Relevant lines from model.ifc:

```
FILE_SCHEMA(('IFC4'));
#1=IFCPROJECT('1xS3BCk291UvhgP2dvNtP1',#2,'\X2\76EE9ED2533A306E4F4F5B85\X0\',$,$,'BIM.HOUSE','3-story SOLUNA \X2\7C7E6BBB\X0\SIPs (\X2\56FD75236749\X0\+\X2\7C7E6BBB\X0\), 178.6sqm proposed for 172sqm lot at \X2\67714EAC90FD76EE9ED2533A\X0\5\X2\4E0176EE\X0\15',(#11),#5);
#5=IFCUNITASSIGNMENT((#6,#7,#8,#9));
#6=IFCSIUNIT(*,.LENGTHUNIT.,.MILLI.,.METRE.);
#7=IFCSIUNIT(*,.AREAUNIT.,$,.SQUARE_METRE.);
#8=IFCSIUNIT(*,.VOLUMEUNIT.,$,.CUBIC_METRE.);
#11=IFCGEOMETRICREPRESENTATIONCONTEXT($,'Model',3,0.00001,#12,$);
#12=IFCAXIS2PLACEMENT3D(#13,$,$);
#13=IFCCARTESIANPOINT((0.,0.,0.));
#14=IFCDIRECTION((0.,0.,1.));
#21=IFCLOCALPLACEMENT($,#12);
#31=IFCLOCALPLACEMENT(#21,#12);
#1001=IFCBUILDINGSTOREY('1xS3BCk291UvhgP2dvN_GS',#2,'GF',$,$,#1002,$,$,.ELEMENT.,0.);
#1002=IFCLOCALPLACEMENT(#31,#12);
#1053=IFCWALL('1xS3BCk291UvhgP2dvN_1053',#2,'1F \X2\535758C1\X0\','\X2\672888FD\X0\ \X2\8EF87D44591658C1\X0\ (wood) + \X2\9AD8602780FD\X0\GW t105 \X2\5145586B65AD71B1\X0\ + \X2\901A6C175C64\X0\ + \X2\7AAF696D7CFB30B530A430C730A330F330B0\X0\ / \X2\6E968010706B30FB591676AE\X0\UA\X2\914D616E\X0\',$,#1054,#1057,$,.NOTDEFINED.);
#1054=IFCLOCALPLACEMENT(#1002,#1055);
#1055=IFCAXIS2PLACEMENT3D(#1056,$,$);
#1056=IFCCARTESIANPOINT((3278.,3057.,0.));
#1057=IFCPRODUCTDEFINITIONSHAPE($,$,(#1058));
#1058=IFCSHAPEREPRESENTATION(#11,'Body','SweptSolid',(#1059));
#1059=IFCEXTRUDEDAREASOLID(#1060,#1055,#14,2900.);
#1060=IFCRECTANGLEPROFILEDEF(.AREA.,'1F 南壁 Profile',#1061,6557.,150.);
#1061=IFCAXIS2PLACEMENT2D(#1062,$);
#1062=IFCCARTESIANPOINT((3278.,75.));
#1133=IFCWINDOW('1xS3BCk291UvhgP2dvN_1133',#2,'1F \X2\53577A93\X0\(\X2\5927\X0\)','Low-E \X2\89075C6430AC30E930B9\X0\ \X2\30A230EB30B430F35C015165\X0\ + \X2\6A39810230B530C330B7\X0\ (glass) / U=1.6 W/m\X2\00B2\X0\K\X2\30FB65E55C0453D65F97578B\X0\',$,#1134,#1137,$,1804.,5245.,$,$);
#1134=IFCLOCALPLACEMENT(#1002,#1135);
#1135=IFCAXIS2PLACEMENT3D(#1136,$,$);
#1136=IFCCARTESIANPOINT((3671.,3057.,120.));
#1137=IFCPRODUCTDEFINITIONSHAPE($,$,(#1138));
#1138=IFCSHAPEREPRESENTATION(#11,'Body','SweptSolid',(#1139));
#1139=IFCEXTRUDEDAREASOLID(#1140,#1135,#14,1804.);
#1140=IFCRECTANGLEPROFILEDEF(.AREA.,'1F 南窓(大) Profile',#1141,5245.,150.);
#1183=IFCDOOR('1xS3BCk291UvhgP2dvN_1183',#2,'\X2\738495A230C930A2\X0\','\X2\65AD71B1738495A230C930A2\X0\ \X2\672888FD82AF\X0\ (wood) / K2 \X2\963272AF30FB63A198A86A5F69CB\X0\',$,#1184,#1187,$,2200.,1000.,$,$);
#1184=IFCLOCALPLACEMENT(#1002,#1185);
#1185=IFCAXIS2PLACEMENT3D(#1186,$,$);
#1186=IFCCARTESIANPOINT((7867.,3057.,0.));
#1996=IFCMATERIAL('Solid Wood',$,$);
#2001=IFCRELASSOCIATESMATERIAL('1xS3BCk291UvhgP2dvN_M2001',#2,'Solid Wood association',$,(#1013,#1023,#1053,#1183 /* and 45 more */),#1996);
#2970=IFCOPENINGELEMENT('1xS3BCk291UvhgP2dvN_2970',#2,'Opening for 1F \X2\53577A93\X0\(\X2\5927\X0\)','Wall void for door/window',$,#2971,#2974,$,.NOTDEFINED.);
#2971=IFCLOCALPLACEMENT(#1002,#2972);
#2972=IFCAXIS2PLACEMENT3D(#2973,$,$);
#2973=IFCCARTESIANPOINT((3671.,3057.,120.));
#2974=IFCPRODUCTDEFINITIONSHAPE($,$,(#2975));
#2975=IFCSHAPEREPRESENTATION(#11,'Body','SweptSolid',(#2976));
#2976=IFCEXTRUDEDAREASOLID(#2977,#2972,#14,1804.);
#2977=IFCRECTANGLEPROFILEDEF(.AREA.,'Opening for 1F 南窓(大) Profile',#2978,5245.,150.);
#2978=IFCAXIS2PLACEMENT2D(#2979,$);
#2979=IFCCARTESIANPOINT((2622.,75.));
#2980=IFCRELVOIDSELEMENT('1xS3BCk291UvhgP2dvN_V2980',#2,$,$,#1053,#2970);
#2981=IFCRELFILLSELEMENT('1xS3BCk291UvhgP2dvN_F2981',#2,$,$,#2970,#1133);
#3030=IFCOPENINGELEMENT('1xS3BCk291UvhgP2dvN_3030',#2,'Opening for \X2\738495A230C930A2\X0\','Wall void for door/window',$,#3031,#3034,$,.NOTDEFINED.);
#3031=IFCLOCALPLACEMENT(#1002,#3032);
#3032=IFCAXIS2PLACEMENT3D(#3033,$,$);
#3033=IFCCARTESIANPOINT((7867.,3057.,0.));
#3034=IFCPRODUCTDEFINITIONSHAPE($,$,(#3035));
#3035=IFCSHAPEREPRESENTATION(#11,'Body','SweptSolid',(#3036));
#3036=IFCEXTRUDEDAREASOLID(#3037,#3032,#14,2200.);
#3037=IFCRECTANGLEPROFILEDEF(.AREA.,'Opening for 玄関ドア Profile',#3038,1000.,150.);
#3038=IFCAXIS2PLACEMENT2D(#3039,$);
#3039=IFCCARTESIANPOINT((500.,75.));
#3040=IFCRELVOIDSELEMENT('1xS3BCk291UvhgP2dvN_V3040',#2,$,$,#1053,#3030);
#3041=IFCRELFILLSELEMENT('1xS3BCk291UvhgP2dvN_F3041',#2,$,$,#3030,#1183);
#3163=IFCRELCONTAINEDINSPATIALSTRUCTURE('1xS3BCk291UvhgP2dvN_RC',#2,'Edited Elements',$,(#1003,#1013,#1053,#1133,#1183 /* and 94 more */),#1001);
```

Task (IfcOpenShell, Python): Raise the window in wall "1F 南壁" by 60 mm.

```python
import numpy as np
import ifcopenshell
import ifcopenshell.api.geometry
import ifcopenshell.util.placement
import ifcopenshell.util.unit

model = ifcopenshell.open("model.ifc")
unit_scale = ifcopenshell.util.unit.calculate_unit_scale(model)

window = model.by_guid("1xS3BCk291UvhgP2dvN_1133")
opening = window.FillsVoids[0].RelatingOpeningElement
dz = 0.06 / unit_scale

shift = np.array([0.0, 0.0, dz])
# The window is not placed relative to its opening, so move both.
for product in (opening, window):
    matrix = ifcopenshell.util.placement.get_local_placement(product.ObjectPlacement)
    matrix[:3, 3] += shift
    ifcopenshell.api.geometry.edit_object_placement(model, product=product, matrix=matrix, is_si=False)

print(f"moved by {dz * unit_scale:+.3f} m")

model.write("model_edited.ifc")
```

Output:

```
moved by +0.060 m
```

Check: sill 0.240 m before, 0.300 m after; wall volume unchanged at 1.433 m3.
